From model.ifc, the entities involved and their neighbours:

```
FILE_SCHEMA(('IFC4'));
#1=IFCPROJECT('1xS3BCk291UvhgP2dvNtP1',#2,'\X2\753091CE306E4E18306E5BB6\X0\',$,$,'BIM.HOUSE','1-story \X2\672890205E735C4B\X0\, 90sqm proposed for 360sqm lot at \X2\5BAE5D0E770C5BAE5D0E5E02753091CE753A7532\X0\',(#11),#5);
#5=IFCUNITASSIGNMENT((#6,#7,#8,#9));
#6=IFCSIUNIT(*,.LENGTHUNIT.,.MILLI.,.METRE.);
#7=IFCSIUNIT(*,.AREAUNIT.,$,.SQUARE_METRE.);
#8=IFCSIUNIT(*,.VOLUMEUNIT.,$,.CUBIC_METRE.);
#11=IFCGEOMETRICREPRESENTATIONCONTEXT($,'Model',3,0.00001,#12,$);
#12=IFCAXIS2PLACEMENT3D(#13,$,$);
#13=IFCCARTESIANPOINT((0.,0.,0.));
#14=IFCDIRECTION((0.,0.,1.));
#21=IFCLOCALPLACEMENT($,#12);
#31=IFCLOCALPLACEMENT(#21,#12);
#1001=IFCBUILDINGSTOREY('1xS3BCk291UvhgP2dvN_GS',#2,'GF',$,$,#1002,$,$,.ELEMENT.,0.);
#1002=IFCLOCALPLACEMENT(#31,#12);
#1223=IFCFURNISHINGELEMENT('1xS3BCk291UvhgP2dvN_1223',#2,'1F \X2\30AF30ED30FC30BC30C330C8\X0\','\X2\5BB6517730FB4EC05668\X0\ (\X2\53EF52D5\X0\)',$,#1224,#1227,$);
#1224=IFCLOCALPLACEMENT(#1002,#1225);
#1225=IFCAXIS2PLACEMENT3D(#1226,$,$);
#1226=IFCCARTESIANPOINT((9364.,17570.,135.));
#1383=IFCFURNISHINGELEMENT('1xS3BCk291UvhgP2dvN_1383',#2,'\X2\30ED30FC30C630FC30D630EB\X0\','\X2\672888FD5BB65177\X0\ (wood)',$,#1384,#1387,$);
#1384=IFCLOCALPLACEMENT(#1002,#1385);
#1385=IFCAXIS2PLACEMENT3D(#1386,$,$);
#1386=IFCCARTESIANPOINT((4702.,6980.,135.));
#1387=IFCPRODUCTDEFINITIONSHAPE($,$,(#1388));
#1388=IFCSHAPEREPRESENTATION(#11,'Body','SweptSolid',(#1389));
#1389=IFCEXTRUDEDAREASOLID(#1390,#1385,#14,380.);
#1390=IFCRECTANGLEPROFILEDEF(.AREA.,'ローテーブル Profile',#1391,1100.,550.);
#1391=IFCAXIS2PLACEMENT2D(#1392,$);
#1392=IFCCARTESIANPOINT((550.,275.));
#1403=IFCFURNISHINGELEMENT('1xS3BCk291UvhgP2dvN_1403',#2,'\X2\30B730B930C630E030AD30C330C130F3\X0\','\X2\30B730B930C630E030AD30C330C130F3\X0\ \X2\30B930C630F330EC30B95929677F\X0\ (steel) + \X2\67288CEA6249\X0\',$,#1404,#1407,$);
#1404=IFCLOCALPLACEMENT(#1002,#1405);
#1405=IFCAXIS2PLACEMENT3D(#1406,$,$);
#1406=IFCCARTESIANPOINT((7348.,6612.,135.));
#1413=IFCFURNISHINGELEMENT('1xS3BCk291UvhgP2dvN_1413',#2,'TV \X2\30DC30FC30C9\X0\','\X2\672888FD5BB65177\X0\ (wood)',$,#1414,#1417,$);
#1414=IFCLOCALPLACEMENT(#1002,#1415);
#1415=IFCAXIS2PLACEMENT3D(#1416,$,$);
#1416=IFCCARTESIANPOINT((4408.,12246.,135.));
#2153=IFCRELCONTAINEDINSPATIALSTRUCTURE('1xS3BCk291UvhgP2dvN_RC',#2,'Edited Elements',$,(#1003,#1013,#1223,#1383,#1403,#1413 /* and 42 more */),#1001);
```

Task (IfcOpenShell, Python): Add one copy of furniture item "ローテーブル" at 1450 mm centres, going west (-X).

```python
import numpy as np
import ifcopenshell
import ifcopenshell.api.geometry
import ifcopenshell.api.root
import ifcopenshell.util.element
import ifcopenshell.util.placement
import ifcopenshell.util.unit

model = ifcopenshell.open("model.ifc")
unit_scale = ifcopenshell.util.unit.calculate_unit_scale(model)


def reuse_history(source, copy):
    """copy_class also copies each property set's owner history, people and application; keep the originals."""
    for rel in copy.IsDefinedBy:
        if rel.is_a("IfcRelDefinesByProperties") and (history := rel.RelatingPropertyDefinition.OwnerHistory):
            rel.RelatingPropertyDefinition.OwnerHistory = source.OwnerHistory
            ifcopenshell.util.element.remove_deep2(model, history)


source = model.by_guid("1xS3BCk291UvhgP2dvN_1383")
base = ifcopenshell.util.placement.get_local_placement(source.ObjectPlacement)
step = np.array([-1.0, 0.0, 0.0]) * 1.45 / unit_scale

for i in range(1, 2):
    copy = ifcopenshell.api.root.copy_class(model, product=source)
    copy.Representation = ifcopenshell.util.element.copy_deep(
        model, source.Representation, exclude=["IfcGeometricRepresentationContext", "IfcRepresentationMap"]
    )
    reuse_history(source, copy)
    matrix = base.copy()
    matrix[:3, 3] += i * step
    print("added at", matrix[:3, 3].round(3) + 0.0)
    ifcopenshell.api.geometry.edit_object_placement(model, product=copy, matrix=matrix, is_si=False)

model.write("model_rev.ifc")
```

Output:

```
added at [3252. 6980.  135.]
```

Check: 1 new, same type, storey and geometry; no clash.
